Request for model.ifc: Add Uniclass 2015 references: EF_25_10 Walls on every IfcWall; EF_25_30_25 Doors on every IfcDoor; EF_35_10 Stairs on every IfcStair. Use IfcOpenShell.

First a look at what the model holds.

```python
import ifcopenshell

model = ifcopenshell.open("model.ifc")
print(model.schema)
print("classifications:", [c.Name for c in model.by_type("IfcClassification")])
for ifc_class in ("IfcDoor", "IfcRoof", "IfcStair", "IfcWall", "IfcWindow"):
    print(ifc_class, len(model.by_type(ifc_class)))
```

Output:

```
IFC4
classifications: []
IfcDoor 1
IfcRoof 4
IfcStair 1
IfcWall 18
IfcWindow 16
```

```python
import ifcopenshell
import ifcopenshell.api.classification

model = ifcopenshell.open("model.ifc")

system = ifcopenshell.api.classification.add_classification(model, classification="Uniclass 2015")

codes = {
    "IfcWall": ("EF_25_10", "Walls"),
    "IfcDoor": ("EF_25_30_25", "Doors"),
    "IfcStair": ("EF_35_10", "Stairs"),
}
for ifc_class, (code, name) in codes.items():
    products = model.by_type(ifc_class)
    ifcopenshell.api.classification.add_reference(
        model, products=products, classification=system, identification=code, name=name
    )
    print(code, len(products))

model.write("model_rev.ifc")
```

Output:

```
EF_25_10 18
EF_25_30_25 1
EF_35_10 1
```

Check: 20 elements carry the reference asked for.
